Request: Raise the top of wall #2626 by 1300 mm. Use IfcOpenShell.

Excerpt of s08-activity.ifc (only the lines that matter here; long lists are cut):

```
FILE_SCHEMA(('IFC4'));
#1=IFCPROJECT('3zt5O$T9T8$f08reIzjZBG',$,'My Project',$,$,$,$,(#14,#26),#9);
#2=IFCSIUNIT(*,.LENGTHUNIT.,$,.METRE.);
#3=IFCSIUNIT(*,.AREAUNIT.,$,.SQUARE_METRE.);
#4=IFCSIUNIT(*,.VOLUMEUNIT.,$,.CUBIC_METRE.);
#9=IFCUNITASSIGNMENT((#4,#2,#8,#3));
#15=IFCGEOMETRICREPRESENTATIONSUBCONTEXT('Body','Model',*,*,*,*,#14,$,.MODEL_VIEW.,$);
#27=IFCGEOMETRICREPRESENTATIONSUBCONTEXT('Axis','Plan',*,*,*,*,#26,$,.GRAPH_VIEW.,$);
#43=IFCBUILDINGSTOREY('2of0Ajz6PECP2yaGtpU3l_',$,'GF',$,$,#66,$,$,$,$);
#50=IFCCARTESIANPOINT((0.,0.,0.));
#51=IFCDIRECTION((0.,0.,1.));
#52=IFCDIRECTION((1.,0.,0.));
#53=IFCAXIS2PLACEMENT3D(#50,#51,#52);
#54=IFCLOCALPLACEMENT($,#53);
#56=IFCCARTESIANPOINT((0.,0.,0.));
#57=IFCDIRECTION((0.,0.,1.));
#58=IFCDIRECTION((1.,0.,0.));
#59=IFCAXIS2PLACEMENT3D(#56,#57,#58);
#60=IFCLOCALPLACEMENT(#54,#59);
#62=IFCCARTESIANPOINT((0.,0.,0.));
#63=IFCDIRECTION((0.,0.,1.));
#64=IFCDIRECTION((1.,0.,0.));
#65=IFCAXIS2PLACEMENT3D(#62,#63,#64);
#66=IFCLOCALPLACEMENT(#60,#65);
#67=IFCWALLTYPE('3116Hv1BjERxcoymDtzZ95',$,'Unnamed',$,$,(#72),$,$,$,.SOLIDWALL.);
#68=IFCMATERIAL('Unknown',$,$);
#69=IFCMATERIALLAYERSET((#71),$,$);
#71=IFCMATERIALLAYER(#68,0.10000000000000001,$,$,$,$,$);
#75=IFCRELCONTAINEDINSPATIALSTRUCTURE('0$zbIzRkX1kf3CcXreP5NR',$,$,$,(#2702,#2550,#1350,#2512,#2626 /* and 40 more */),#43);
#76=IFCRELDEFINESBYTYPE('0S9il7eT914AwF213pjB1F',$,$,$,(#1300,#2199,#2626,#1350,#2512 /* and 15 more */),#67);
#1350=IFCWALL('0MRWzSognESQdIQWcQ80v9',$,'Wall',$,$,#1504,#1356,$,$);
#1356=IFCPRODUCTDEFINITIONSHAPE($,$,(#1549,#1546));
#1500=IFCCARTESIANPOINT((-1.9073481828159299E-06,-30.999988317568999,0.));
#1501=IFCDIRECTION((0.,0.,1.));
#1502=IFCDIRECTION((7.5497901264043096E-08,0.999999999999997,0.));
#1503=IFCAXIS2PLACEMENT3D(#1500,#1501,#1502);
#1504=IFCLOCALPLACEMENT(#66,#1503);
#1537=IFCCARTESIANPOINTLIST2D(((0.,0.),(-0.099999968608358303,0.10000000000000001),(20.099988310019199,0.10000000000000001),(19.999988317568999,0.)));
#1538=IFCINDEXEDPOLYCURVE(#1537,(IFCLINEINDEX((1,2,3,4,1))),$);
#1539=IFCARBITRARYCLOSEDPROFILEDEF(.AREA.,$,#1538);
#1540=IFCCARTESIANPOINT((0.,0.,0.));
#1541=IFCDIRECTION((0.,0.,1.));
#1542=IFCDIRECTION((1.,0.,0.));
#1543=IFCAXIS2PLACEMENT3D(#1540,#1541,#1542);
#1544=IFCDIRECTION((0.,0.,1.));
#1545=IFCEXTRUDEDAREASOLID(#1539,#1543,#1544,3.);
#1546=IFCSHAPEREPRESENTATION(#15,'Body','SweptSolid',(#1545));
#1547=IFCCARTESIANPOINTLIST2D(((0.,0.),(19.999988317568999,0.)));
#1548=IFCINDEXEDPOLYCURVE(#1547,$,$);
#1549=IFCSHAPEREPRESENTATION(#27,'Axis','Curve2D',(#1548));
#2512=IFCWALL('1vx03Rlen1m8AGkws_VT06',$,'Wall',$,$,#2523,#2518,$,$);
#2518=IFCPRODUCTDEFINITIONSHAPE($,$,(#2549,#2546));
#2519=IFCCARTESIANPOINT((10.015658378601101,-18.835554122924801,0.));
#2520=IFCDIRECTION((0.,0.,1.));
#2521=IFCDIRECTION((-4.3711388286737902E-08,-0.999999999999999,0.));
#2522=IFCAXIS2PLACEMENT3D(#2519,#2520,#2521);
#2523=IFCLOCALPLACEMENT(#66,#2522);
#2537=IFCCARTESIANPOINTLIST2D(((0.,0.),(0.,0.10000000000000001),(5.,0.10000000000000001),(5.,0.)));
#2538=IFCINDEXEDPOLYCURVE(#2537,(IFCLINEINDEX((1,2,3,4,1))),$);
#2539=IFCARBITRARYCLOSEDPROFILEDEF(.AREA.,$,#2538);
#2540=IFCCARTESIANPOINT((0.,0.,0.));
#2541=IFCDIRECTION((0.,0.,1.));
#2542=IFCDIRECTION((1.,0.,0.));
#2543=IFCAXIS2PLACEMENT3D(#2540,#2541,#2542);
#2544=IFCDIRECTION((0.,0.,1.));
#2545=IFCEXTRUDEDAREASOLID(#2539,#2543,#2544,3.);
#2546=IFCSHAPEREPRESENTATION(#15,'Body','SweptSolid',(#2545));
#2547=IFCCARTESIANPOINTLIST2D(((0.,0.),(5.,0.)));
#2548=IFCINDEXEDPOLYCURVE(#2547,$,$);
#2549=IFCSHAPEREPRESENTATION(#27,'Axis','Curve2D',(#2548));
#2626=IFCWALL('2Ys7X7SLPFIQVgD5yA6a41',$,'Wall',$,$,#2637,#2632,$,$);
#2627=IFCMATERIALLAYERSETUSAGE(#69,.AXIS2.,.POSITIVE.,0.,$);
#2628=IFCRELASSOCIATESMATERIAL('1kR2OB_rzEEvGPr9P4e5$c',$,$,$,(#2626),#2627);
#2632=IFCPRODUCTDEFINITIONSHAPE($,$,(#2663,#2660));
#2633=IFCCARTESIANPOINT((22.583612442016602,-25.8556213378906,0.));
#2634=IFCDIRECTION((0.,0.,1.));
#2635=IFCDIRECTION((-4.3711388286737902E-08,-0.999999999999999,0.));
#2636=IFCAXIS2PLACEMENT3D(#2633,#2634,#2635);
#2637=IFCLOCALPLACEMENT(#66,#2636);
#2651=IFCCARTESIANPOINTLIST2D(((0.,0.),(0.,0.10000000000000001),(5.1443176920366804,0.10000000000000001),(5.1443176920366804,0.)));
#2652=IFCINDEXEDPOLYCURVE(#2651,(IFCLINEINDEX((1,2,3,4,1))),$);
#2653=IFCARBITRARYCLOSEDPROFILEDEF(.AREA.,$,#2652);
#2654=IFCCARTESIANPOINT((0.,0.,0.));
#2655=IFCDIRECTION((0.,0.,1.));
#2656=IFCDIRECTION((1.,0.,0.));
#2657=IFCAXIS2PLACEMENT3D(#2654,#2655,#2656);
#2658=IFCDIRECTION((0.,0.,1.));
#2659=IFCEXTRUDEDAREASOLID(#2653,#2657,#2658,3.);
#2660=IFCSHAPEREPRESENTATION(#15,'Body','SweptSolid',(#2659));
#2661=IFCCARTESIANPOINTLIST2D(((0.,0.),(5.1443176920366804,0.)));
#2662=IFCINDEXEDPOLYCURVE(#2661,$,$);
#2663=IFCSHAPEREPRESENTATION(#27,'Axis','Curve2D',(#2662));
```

```python
import ifcopenshell
import ifcopenshell.geom
import ifcopenshell.util.representation
import ifcopenshell.util.shape

model = ifcopenshell.open("s08-activity.ifc")
settings = ifcopenshell.geom.settings()


def volume(element):
    """Net volume in cubic metres, openings subtracted."""
    shape = ifcopenshell.geom.create_shape(settings, element)
    return ifcopenshell.util.shape.get_volume(shape.geometry)


wall = model.by_guid("2Ys7X7SLPFIQVgD5yA6a41")
before = volume(wall)

body = ifcopenshell.util.representation.get_representation(wall, "Model", "Body")
solid = body.Items[0]
old_height = solid.Depth
solid.Depth += 1.3
after = volume(wall)

print(f"height {old_height:g} -> {solid.Depth:g}, volume {before:.3f} -> {after:.3f} m3")

model.write("s08-activity_rev.ifc")
```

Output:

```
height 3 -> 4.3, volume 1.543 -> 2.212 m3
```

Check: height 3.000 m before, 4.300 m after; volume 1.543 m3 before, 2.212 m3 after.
